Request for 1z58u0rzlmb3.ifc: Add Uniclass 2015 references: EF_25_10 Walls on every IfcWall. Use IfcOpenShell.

First a look at what the model holds.

```python
import ifcopenshell

model = ifcopenshell.open("1z58u0rzlmb3.ifc")
print(model.schema)
print("classifications:", [c.Name for c in model.by_type("IfcClassification")])
for ifc_class in ("IfcDoor", "IfcRoof", "IfcStair", "IfcWall", "IfcWindow"):
    print(ifc_class, len(model.by_type(ifc_class)))
```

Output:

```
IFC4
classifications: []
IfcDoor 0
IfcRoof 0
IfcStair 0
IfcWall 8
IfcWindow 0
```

```python
import ifcopenshell
import ifcopenshell.api.classification

model = ifcopenshell.open("1z58u0rzlmb3.ifc")

system = ifcopenshell.api.classification.add_classification(model, classification="Uniclass 2015")

codes = {
    "IfcWall": ("EF_25_10", "Walls"),
}
for ifc_class, (code, name) in codes.items():
    products = model.by_type(ifc_class)
    ifcopenshell.api.classification.add_reference(
        model, products=products, classification=system, identification=code, name=name
    )
    print(code, len(products))

model.write("1z58u0rzlmb3_rev.ifc")
```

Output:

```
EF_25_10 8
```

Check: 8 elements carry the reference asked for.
